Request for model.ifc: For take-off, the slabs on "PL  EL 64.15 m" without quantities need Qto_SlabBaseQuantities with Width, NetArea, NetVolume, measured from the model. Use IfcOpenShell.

First a look at what the model holds.

```python
import ifcopenshell
import ifcopenshell.util.element
import ifcopenshell.util.unit

model = ifcopenshell.open("model.ifc")
print(model.schema)
for unit_type in ("LENGTHUNIT", "AREAUNIT", "VOLUMEUNIT"):
    print(unit_type, ifcopenshell.util.unit.calculate_unit_scale(model, unit_type))
storey = next(s for s in model.by_type("IfcBuildingStorey") if s.Name == "PL  EL 64.15 m")
slabs = [e for e in ifcopenshell.util.element.get_decomposition(storey) if e.is_a("IfcSlab")]
for e in sorted(slabs, key=lambda e: e.id()):
    print(e.id(), e.is_a(), e.Name, list(ifcopenshell.util.element.get_psets(e, qtos_only=True)), sep=" | ")
```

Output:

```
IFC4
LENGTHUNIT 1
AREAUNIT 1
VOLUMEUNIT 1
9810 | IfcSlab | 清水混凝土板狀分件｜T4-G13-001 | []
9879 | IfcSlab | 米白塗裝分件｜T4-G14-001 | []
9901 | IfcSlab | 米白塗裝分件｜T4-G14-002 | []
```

```python
import ifcopenshell
import ifcopenshell.api.pset
import ifcopenshell.geom
import ifcopenshell.util.element
import ifcopenshell.util.shape
import ifcopenshell.util.unit

model = ifcopenshell.open("model.ifc")
unit_scale = ifcopenshell.util.unit.calculate_unit_scale(model)
area_scale = ifcopenshell.util.unit.calculate_unit_scale(model, "AREAUNIT")
volume_scale = ifcopenshell.util.unit.calculate_unit_scale(model, "VOLUMEUNIT")
settings = ifcopenshell.geom.settings()

storey = next(s for s in model.by_type("IfcBuildingStorey") if s.Name == "PL  EL 64.15 m")
slabs = [e for e in ifcopenshell.util.element.get_decomposition(storey) if e.is_a("IfcSlab")]

for e in sorted(slabs, key=lambda e: e.id()):
    if ifcopenshell.util.element.get_psets(e, qtos_only=True, should_inherit=False):
        continue
    # Geometry comes back in metres, in the element's own axes.
    shape = ifcopenshell.geom.create_shape(settings, e)
    values = {
        "Width": ifcopenshell.util.shape.get_z(shape.geometry) / unit_scale,
        "NetArea": ifcopenshell.util.shape.get_footprint_area(shape.geometry) / area_scale,
        "NetVolume": ifcopenshell.util.shape.get_volume(shape.geometry) / volume_scale,
    }
    qto = ifcopenshell.api.pset.add_qto(model, product=e, name="Qto_SlabBaseQuantities")
    ifcopenshell.api.pset.edit_qto(model, qto=qto, properties=values)
    print(e.id(), {k: round(v, 3) for k, v in values.items()})

model.write("model-out.ifc")
```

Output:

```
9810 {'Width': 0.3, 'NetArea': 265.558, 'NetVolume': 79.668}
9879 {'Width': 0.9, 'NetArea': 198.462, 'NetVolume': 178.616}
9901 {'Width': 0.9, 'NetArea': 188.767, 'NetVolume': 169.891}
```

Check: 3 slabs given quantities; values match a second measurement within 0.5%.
